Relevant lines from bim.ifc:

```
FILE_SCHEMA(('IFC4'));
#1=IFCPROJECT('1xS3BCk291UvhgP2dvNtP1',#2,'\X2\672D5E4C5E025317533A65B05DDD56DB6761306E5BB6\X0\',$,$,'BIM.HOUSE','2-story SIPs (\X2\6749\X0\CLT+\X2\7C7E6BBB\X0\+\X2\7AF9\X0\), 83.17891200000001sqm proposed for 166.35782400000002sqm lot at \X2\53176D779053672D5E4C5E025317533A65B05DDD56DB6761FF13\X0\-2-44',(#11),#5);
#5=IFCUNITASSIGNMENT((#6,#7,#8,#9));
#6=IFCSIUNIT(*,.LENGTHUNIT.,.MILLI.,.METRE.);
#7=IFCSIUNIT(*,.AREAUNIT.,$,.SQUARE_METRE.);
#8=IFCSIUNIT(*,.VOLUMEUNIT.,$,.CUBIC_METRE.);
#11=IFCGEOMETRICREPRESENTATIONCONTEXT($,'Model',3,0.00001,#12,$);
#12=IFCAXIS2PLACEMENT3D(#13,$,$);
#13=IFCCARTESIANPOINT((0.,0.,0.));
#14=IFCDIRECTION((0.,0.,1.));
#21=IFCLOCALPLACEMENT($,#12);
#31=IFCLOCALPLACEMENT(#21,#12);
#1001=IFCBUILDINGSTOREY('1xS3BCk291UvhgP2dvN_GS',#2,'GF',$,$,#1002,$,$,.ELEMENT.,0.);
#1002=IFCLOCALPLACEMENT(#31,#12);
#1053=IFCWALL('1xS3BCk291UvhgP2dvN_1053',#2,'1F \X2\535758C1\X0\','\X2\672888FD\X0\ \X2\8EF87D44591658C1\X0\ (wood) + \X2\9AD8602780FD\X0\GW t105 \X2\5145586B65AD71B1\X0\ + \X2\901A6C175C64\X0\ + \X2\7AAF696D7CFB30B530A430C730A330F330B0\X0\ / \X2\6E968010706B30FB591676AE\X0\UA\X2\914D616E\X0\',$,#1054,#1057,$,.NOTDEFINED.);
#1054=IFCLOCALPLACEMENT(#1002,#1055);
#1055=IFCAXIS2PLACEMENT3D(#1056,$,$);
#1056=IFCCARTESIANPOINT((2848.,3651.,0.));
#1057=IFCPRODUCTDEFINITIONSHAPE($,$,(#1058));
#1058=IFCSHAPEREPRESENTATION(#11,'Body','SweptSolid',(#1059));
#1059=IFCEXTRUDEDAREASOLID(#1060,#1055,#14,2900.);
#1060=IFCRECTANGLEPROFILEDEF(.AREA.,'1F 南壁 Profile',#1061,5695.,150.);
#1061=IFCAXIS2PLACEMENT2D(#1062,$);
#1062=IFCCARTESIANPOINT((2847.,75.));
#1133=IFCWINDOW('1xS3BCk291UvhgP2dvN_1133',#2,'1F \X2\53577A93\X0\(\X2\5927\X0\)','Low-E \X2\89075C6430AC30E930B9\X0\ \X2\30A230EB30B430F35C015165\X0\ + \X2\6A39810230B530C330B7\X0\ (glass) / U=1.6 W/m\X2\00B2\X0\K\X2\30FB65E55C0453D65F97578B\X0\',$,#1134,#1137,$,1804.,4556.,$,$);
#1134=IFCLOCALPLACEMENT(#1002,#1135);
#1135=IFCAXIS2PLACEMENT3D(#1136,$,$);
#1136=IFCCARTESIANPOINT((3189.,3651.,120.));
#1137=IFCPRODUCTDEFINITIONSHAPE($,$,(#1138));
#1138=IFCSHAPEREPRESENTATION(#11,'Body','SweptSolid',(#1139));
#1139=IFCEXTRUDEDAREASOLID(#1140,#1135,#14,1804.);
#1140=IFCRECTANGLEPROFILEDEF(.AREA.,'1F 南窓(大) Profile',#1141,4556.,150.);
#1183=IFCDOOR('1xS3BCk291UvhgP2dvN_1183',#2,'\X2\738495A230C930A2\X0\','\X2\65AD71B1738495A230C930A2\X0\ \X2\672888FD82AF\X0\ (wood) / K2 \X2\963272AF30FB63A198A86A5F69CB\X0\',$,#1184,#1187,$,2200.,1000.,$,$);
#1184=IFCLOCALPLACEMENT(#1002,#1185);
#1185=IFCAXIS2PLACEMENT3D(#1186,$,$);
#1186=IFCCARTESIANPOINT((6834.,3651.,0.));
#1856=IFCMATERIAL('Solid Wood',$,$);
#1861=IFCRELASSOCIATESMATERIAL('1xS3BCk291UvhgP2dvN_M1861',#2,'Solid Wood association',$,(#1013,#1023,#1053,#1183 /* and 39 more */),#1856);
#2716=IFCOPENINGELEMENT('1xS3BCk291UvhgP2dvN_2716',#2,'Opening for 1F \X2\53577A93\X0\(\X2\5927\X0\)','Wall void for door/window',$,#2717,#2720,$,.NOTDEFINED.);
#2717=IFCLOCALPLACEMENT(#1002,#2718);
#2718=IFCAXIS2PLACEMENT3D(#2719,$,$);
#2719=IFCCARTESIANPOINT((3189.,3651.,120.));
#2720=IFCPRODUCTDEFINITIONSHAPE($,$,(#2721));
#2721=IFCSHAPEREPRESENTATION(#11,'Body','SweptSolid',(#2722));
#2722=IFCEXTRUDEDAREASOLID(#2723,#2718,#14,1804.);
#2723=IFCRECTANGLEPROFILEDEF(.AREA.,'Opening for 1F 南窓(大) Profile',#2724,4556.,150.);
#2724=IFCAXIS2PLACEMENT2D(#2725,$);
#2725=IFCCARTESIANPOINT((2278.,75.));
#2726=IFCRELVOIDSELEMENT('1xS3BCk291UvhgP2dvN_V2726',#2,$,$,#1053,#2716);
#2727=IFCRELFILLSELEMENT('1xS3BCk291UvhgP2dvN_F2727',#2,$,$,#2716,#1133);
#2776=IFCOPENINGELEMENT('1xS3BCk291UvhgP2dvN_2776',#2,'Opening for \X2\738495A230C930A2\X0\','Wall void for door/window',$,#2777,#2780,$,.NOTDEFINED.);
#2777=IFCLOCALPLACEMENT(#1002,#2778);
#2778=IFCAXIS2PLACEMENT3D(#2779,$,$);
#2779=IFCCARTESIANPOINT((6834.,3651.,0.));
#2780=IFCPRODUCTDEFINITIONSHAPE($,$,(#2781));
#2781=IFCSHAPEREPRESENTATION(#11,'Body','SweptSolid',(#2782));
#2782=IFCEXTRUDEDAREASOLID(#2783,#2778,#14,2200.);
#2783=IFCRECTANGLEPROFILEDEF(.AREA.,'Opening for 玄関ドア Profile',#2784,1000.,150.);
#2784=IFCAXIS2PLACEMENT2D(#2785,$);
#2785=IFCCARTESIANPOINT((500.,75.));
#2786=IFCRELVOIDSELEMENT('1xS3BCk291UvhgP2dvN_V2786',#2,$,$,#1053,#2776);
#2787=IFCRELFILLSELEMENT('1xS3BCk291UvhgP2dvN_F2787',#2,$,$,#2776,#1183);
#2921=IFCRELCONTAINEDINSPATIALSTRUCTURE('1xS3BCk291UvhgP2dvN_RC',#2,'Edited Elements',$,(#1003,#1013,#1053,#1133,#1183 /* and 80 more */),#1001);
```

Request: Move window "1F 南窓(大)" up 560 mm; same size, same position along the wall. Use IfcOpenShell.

```python
import numpy as np
import ifcopenshell
import ifcopenshell.api.geometry
import ifcopenshell.util.placement
import ifcopenshell.util.unit

model = ifcopenshell.open("bim.ifc")
unit_scale = ifcopenshell.util.unit.calculate_unit_scale(model)

window = model.by_id(1133)
opening = window.FillsVoids[0].RelatingOpeningElement
dz = 0.56 / unit_scale

shift = np.array([0.0, 0.0, dz])
# The window is not placed relative to its opening, so move both.
for product in (opening, window):
    matrix = ifcopenshell.util.placement.get_local_placement(product.ObjectPlacement)
    matrix[:3, 3] += shift
    ifcopenshell.api.geometry.edit_object_placement(model, product=product, matrix=matrix, is_si=False)

print(f"moved by {dz * unit_scale:+.3f} m")

model.write("bim-out.ifc")
```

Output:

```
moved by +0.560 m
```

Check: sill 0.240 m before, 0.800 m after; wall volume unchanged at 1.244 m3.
